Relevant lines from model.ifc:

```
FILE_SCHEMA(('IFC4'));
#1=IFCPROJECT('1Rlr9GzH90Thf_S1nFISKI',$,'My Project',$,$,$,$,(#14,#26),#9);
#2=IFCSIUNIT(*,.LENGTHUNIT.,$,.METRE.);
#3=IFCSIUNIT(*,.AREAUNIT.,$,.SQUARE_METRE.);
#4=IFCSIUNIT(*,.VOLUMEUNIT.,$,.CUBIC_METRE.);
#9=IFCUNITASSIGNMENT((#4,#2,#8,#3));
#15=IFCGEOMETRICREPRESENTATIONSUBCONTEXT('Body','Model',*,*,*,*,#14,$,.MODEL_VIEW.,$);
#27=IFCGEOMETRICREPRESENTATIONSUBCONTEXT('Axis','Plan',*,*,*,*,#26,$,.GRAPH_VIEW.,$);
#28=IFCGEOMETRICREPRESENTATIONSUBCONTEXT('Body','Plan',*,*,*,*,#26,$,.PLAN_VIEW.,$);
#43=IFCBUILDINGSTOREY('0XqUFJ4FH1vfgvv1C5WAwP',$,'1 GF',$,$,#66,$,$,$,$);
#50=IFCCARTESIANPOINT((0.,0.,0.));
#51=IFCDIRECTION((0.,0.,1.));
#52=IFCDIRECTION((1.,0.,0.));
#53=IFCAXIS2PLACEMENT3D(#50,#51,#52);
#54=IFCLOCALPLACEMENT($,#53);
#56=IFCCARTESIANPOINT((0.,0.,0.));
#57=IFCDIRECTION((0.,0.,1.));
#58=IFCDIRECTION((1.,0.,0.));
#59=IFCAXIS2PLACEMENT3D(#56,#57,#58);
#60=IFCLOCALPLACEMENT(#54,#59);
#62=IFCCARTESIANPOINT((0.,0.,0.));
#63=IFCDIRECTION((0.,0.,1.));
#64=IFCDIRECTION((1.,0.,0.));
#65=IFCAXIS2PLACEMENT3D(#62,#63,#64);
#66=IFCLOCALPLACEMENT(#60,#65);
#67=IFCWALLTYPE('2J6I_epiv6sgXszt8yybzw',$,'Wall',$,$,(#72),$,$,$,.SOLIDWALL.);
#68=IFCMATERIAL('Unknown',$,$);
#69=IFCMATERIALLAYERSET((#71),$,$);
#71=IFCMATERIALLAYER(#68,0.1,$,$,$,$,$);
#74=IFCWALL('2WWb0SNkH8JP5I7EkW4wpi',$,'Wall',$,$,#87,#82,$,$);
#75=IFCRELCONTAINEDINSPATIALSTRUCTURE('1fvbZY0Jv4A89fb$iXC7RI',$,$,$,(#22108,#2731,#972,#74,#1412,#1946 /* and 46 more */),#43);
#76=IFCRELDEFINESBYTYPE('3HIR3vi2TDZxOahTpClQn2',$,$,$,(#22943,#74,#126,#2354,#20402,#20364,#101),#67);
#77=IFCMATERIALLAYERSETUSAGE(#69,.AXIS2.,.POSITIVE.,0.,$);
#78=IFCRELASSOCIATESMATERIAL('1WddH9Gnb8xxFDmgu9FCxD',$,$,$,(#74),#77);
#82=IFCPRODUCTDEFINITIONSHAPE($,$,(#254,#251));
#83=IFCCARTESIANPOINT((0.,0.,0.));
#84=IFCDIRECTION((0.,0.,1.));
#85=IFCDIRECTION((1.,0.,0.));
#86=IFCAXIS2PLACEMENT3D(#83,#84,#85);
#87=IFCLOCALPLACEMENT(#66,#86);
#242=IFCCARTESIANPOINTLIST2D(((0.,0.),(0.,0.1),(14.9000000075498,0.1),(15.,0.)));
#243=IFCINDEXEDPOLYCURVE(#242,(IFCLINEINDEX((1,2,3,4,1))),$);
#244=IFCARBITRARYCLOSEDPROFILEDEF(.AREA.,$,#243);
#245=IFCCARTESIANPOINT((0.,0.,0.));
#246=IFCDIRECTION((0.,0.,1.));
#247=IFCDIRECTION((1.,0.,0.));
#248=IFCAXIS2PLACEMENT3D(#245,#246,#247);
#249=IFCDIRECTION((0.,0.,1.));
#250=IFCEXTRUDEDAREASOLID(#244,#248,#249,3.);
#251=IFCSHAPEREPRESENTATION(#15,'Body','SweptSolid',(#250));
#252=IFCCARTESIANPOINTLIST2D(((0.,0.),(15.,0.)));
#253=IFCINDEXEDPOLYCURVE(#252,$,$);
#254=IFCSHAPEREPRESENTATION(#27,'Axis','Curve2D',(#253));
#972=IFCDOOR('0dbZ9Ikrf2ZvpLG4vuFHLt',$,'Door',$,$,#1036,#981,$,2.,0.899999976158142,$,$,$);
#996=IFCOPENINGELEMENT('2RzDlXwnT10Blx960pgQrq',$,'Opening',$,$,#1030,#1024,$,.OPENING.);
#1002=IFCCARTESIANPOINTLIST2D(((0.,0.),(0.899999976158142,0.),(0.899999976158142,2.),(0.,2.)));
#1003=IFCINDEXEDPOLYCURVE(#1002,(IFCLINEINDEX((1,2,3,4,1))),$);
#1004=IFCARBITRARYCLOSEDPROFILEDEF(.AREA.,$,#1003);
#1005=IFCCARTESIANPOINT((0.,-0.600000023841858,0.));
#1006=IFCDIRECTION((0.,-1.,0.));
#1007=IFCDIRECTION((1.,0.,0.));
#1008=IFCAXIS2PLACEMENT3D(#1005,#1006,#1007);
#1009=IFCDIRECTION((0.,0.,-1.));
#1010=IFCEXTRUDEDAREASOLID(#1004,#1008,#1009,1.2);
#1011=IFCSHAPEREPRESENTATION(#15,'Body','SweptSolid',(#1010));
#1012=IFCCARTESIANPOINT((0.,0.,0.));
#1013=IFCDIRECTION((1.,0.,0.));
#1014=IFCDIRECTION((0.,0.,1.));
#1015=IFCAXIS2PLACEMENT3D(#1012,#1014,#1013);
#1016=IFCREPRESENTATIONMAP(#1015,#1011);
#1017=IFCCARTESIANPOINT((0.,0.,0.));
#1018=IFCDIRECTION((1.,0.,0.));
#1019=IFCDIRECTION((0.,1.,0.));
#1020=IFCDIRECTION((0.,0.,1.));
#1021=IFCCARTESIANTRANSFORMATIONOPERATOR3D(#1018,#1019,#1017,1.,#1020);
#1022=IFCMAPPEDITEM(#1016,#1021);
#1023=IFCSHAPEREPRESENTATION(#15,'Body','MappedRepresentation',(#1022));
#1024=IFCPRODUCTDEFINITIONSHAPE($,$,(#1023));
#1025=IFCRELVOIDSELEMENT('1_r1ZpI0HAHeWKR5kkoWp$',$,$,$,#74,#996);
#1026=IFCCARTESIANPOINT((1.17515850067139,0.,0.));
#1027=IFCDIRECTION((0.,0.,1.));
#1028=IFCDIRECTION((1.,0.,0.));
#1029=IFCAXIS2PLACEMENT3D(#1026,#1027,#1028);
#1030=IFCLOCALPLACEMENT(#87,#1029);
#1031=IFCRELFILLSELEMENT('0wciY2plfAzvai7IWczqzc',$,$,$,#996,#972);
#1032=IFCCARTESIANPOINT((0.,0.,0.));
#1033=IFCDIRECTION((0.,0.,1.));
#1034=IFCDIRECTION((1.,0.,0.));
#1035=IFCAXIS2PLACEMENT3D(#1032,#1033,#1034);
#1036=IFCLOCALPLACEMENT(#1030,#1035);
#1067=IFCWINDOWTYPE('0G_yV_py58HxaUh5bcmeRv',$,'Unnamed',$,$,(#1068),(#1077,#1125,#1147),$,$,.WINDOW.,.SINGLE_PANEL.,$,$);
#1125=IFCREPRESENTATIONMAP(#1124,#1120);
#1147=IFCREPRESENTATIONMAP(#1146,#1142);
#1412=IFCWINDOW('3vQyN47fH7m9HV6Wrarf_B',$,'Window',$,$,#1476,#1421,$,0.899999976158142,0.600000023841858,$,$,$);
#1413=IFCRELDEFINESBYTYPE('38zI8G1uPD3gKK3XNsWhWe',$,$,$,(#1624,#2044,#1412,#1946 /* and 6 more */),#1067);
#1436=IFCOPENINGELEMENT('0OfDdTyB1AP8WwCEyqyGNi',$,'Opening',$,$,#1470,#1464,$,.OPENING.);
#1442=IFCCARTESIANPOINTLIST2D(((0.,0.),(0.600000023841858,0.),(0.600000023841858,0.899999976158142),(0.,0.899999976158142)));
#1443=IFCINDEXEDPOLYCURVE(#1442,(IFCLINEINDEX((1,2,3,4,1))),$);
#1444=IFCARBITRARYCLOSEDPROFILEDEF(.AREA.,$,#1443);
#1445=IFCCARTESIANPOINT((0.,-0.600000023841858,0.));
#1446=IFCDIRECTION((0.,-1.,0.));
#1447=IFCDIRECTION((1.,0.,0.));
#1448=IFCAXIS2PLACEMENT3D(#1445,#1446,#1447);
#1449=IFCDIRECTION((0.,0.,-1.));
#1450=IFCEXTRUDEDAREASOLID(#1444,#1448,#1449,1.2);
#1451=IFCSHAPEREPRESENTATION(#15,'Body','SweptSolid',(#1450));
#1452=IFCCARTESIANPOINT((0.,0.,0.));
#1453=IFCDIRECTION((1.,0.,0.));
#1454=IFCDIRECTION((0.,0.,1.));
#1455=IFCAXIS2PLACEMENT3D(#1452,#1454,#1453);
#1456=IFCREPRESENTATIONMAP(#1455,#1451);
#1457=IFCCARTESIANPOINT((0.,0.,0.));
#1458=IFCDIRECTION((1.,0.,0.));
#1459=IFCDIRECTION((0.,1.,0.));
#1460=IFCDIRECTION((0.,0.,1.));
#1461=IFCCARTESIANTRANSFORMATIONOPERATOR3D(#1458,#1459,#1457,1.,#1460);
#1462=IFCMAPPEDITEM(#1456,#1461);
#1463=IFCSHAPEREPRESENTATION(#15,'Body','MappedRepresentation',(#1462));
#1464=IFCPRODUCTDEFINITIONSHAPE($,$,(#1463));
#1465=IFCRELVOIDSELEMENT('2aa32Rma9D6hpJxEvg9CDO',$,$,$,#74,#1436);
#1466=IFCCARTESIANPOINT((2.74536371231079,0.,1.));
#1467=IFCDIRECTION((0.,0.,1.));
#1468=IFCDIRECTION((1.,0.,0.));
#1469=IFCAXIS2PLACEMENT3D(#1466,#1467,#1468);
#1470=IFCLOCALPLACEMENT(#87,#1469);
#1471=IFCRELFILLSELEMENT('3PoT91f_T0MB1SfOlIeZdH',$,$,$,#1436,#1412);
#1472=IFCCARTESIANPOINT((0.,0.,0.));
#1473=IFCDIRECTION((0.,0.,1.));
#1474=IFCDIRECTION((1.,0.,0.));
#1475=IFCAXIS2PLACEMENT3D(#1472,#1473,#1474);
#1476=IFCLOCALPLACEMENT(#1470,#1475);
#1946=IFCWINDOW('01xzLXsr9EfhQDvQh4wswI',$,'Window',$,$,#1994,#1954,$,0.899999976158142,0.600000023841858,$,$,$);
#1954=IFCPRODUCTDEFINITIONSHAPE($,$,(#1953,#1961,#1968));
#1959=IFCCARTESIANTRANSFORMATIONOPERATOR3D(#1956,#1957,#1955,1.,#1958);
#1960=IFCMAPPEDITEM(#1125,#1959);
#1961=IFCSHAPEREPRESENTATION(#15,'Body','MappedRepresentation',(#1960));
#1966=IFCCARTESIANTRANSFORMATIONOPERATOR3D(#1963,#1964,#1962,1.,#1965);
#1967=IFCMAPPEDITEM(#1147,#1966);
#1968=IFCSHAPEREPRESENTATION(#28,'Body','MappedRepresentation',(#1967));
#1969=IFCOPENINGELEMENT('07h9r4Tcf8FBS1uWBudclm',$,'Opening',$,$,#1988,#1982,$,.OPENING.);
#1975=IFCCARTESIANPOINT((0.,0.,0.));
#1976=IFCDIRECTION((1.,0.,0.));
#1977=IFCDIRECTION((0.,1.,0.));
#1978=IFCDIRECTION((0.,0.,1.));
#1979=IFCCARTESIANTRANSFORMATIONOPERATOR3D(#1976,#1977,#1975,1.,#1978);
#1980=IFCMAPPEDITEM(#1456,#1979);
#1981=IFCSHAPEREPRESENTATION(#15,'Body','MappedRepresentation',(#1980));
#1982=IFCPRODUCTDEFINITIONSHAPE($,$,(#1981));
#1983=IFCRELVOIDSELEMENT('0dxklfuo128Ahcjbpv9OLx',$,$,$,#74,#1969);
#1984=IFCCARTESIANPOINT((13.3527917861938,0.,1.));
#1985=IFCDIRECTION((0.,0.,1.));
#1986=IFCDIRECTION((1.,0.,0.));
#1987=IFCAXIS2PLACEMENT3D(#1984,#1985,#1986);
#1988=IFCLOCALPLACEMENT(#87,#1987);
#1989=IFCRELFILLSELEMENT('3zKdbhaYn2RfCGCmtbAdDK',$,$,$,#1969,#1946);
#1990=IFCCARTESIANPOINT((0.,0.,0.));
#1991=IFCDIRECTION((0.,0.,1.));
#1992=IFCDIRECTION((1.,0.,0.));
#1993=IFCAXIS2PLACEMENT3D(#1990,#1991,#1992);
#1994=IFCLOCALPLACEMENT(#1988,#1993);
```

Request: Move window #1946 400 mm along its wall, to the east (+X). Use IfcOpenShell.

```python
import ifcopenshell
import ifcopenshell.api.geometry
import ifcopenshell.util.placement

model = ifcopenshell.open("model.ifc")

window = model.by_guid("01xzLXsr9EfhQDvQh4wswI")
opening = window.FillsVoids[0].RelatingOpeningElement
wall = opening.VoidsElements[0].RelatingBuildingElement

wall_matrix = ifcopenshell.util.placement.get_local_placement(wall.ObjectPlacement)
shift = wall_matrix[:3, 0] * 0.4
before = ifcopenshell.util.placement.get_local_placement(window.ObjectPlacement)[:3, 3].copy()

# The window is placed relative to its opening, so it follows when the opening moves.
matrix = ifcopenshell.util.placement.get_local_placement(opening.ObjectPlacement)
matrix[:3, 3] += shift
ifcopenshell.api.geometry.edit_object_placement(
    model, product=opening, matrix=matrix, is_si=False, should_transform_children=True
)

after = ifcopenshell.util.placement.get_local_placement(window.ObjectPlacement)[:3, 3]
print("window moved by", (after - before).round(3) + 0.0)

model.write("model-out.ifc")
```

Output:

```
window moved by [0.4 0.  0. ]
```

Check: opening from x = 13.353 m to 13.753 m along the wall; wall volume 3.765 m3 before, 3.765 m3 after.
